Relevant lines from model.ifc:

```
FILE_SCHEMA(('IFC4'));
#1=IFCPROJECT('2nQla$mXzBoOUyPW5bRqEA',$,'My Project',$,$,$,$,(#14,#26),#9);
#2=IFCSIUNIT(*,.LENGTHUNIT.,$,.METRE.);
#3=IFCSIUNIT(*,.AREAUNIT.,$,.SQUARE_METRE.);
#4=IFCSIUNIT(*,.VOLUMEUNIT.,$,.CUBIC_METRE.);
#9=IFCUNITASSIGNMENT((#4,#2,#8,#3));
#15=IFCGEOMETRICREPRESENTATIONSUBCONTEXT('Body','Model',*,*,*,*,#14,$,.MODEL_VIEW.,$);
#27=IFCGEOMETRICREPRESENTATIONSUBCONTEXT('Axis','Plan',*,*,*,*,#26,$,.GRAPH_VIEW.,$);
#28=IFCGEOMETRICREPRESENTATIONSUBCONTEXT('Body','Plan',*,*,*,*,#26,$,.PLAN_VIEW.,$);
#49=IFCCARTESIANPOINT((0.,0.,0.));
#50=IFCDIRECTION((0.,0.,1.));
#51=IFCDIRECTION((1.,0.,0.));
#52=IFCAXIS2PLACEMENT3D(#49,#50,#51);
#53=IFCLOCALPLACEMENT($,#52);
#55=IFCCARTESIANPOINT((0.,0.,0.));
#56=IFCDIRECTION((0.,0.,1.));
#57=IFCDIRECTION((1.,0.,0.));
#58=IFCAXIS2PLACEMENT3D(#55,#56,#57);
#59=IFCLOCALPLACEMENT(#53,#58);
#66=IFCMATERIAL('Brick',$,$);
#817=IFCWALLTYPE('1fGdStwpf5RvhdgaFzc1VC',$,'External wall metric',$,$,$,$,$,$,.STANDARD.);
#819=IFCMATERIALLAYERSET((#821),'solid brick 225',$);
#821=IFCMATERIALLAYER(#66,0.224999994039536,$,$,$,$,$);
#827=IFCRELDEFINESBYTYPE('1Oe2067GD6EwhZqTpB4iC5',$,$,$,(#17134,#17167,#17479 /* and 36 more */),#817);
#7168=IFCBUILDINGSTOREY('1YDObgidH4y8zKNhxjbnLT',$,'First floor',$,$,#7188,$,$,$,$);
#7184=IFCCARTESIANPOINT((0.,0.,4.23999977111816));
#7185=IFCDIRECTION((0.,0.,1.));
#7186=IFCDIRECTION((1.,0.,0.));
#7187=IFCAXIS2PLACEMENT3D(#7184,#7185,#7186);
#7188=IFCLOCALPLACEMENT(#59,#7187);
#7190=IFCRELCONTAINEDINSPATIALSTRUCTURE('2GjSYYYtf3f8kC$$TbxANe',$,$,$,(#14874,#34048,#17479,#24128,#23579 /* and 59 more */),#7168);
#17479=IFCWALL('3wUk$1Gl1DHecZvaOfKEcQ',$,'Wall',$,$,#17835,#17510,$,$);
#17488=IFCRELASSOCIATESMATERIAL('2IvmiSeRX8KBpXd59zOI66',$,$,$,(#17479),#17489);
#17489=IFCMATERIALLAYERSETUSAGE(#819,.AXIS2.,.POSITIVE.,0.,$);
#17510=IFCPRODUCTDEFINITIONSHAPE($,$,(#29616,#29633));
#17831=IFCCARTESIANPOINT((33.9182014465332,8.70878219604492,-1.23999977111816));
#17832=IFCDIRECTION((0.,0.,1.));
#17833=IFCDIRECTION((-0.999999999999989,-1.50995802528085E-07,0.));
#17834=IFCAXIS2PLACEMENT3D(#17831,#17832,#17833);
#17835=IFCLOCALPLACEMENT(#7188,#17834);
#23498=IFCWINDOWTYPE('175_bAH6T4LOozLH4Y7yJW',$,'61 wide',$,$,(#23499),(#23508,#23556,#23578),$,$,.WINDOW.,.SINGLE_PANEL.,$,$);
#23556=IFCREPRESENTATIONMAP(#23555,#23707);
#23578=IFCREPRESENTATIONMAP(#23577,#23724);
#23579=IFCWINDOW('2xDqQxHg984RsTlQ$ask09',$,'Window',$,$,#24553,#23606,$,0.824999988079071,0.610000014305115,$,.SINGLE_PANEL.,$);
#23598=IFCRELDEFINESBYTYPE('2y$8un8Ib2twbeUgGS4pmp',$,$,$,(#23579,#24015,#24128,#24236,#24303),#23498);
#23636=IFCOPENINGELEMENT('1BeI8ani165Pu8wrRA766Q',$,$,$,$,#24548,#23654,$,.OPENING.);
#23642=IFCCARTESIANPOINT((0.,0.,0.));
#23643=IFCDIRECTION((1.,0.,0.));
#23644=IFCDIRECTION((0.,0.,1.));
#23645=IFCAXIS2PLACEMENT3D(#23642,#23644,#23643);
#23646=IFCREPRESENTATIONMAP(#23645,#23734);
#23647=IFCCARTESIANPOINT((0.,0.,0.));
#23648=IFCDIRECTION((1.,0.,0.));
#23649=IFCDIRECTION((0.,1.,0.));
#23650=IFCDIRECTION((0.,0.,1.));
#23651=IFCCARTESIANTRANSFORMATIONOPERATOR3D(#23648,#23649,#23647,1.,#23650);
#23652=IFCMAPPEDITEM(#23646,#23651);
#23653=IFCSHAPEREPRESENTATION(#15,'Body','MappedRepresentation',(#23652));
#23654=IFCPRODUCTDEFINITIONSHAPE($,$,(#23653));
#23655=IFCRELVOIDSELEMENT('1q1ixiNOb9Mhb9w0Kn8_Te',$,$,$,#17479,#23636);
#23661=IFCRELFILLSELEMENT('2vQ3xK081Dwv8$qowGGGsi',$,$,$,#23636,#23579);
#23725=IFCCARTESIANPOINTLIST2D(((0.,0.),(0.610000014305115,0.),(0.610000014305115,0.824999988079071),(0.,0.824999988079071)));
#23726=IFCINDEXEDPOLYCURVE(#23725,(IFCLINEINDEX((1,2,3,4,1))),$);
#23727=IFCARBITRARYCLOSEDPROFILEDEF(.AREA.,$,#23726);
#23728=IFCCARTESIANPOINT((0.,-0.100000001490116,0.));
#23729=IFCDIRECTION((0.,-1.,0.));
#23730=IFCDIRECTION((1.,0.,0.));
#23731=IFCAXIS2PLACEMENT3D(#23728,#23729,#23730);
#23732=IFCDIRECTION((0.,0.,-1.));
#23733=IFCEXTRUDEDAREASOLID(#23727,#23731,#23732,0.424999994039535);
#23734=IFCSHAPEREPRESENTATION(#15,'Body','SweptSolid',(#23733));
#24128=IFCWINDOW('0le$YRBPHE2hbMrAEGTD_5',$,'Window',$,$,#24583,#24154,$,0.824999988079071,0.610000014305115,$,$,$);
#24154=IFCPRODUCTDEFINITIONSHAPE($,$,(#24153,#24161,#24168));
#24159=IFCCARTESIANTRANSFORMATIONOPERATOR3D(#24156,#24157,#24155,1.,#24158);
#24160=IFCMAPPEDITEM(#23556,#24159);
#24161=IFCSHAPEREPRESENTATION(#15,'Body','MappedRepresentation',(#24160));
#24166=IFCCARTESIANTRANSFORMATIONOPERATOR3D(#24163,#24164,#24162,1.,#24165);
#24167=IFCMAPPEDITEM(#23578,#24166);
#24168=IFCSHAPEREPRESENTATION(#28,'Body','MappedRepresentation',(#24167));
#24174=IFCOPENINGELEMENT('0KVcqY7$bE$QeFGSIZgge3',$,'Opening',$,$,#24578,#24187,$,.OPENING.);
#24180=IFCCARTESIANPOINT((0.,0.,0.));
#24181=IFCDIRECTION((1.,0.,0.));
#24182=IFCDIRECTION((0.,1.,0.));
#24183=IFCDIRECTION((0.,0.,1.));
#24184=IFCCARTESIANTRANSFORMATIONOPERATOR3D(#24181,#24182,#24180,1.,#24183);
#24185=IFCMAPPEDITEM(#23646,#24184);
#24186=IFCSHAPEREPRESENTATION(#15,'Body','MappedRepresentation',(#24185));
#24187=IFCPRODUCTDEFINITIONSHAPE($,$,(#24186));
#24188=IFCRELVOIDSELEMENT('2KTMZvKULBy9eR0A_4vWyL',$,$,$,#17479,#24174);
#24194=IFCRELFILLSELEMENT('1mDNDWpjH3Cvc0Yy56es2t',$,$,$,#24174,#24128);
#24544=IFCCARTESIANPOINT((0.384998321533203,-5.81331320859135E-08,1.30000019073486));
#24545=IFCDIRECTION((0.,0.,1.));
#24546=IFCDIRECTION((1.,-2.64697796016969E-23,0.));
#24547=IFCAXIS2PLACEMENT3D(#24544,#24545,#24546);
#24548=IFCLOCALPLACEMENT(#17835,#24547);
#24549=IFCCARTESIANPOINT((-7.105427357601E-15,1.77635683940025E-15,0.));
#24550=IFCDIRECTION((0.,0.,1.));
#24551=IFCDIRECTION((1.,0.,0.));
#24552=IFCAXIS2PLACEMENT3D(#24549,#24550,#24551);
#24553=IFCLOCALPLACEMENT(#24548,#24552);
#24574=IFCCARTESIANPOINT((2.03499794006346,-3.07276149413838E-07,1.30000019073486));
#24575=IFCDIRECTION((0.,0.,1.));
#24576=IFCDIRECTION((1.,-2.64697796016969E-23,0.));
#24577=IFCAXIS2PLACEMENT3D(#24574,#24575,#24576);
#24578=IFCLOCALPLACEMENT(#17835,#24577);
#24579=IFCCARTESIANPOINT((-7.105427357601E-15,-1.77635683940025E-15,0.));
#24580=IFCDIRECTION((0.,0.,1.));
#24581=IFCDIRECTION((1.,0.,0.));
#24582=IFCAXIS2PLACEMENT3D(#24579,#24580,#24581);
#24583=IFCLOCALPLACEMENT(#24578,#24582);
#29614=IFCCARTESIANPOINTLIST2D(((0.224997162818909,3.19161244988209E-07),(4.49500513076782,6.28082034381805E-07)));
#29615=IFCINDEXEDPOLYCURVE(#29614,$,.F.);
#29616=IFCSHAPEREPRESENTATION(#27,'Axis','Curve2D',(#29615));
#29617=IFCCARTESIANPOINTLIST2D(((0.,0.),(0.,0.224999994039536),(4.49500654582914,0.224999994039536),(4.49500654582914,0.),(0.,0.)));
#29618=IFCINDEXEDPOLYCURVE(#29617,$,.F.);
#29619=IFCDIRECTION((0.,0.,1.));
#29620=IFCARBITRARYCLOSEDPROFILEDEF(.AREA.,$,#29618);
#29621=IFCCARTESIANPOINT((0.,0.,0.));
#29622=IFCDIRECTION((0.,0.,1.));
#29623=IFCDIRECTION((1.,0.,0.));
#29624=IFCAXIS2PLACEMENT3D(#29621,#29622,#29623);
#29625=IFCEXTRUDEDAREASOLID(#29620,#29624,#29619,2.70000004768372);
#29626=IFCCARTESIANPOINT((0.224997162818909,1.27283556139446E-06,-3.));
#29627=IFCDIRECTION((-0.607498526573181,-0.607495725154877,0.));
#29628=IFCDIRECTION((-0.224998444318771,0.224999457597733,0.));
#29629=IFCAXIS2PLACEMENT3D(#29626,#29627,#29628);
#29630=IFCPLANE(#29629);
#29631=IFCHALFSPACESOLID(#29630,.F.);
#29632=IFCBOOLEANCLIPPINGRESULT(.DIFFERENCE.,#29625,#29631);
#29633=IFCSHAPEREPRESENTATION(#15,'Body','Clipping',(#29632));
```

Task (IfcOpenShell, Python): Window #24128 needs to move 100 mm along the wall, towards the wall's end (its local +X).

```python
import ifcopenshell
import ifcopenshell.api.geometry
import ifcopenshell.util.placement
import ifcopenshell.util.unit

model = ifcopenshell.open("model.ifc")
unit_scale = ifcopenshell.util.unit.calculate_unit_scale(model)

window = model.by_guid("0le$YRBPHE2hbMrAEGTD_5")
opening = window.FillsVoids[0].RelatingOpeningElement
wall = opening.VoidsElements[0].RelatingBuildingElement

wall_matrix = ifcopenshell.util.placement.get_local_placement(wall.ObjectPlacement)
shift = wall_matrix[:3, 0] * 0.1 / unit_scale
before = ifcopenshell.util.placement.get_local_placement(window.ObjectPlacement)[:3, 3].copy()

# The window is placed relative to its opening, so it follows when the opening moves.
matrix = ifcopenshell.util.placement.get_local_placement(opening.ObjectPlacement)
matrix[:3, 3] += shift
ifcopenshell.api.geometry.edit_object_placement(
    model, product=opening, matrix=matrix, is_si=False, should_transform_children=True
)

after = ifcopenshell.util.placement.get_local_placement(window.ObjectPlacement)[:3, 3]
print("window moved by", (after - before).round(3) + 0.0)

model.write("model_updated.ifc")
```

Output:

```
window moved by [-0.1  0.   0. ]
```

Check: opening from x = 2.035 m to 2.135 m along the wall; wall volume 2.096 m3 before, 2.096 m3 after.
